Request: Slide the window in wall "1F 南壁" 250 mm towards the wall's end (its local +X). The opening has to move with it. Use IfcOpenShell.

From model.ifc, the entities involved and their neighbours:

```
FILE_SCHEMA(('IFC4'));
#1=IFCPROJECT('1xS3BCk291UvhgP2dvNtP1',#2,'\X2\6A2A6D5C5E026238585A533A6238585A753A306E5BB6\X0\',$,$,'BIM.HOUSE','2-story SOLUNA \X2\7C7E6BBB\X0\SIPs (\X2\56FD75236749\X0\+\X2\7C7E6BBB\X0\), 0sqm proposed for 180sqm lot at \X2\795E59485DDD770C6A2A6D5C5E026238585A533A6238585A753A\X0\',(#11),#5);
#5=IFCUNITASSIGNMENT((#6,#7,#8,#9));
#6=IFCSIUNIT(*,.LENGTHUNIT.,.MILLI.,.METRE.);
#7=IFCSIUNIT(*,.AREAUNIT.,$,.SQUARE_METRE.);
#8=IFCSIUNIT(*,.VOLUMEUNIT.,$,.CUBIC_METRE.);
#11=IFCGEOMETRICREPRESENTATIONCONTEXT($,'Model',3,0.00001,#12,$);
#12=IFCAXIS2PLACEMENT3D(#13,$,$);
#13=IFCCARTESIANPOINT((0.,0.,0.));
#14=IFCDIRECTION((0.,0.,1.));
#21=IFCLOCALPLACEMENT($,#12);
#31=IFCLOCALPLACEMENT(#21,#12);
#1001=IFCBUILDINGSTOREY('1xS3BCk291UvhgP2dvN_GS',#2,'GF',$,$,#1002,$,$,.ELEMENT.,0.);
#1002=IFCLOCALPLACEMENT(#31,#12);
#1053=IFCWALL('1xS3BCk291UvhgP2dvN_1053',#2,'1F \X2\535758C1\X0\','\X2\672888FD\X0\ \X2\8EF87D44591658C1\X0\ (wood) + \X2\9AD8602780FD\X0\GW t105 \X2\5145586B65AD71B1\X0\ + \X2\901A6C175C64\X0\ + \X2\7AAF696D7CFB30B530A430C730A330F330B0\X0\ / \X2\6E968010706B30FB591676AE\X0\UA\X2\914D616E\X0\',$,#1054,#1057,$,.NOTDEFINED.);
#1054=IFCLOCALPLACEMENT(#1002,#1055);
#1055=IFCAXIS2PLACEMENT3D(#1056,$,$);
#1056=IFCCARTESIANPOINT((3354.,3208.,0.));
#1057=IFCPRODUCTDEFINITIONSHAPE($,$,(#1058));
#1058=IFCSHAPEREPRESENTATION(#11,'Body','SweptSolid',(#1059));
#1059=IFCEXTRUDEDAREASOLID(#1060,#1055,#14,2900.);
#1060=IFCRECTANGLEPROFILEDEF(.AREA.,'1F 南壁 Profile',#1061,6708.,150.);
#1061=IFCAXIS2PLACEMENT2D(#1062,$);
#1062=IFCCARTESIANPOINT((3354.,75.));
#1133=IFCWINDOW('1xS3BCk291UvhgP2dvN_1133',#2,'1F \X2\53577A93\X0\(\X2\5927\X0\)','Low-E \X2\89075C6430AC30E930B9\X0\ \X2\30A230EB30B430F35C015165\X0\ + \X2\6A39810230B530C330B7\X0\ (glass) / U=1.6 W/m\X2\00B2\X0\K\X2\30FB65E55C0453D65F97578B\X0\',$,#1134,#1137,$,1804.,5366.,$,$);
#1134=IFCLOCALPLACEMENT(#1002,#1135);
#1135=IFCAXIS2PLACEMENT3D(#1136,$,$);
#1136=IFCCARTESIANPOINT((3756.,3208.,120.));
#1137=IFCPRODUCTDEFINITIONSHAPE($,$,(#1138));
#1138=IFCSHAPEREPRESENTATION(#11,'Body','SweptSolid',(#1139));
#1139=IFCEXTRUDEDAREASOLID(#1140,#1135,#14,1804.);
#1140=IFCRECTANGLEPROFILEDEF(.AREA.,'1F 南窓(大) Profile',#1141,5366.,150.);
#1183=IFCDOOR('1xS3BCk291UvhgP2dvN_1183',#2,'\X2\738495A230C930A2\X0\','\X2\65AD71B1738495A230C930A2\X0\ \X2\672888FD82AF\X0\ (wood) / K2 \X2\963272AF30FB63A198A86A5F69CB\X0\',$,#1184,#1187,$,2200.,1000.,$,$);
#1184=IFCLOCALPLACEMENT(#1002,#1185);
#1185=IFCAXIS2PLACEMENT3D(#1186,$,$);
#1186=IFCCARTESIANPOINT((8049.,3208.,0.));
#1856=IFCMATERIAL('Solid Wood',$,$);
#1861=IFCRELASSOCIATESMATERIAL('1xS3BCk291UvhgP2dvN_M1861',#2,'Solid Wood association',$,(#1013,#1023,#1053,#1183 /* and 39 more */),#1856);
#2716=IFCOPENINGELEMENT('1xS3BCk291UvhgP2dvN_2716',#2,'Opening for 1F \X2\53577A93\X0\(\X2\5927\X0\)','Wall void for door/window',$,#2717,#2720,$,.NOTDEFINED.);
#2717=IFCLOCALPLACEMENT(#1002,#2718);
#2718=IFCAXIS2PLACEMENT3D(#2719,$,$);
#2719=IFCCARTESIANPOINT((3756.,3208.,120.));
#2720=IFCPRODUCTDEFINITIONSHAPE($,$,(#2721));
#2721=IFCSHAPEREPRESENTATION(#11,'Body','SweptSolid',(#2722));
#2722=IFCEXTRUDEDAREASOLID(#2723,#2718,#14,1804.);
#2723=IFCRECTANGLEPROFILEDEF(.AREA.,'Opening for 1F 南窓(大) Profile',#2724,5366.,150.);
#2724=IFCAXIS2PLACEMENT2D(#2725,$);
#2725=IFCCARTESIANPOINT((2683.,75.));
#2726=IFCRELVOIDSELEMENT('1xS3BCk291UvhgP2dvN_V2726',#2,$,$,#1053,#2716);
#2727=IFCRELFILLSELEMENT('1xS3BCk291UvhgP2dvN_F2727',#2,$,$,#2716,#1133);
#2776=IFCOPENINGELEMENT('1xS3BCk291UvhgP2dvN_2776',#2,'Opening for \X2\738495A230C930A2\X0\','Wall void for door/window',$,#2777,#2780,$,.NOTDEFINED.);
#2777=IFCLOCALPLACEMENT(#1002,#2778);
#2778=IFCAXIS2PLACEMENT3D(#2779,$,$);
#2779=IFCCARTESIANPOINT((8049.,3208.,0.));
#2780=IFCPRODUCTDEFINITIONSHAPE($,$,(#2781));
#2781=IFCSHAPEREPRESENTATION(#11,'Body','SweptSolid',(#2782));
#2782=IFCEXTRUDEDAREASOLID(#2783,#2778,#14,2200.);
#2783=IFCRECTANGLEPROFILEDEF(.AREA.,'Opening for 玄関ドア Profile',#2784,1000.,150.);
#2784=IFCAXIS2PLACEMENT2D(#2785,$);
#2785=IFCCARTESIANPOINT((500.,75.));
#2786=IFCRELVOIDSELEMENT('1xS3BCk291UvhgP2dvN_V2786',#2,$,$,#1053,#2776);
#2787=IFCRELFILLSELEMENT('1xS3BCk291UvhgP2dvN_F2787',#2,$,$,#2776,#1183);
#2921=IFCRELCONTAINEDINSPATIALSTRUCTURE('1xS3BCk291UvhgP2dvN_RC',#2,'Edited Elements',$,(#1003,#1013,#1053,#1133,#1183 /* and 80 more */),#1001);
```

```python
import ifcopenshell
import ifcopenshell.api.geometry
import ifcopenshell.util.placement

model = ifcopenshell.open("model.ifc")

window = model.by_guid("1xS3BCk291UvhgP2dvN_1133")
opening = window.FillsVoids[0].RelatingOpeningElement
wall = opening.VoidsElements[0].RelatingBuildingElement

wall_matrix = ifcopenshell.util.placement.get_local_placement(wall.ObjectPlacement)
shift = wall_matrix[:3, 0] * 250.0
before = ifcopenshell.util.placement.get_local_placement(window.ObjectPlacement)[:3, 3].copy()

# The window is not placed relative to its opening, so move both.
for product in (opening, window):
    matrix = ifcopenshell.util.placement.get_local_placement(product.ObjectPlacement)
    matrix[:3, 3] += shift
    ifcopenshell.api.geometry.edit_object_placement(model, product=product, matrix=matrix, is_si=False)

after = ifcopenshell.util.placement.get_local_placement(window.ObjectPlacement)[:3, 3]
print("window moved by", (after - before).round(3) + 0.0)

model.write("model_v2.ifc")
```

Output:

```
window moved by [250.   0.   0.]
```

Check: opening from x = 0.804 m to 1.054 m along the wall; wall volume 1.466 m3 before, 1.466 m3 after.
